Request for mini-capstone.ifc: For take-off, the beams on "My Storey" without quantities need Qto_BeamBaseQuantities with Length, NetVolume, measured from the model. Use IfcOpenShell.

First a look at what the model holds.

```python
import ifcopenshell
import ifcopenshell.util.element
import ifcopenshell.util.unit

model = ifcopenshell.open("mini-capstone.ifc")
print(model.schema)
for unit_type in ("LENGTHUNIT", "AREAUNIT", "VOLUMEUNIT"):
    print(unit_type, ifcopenshell.util.unit.calculate_unit_scale(model, unit_type))
storey = next(s for s in model.by_type("IfcBuildingStorey") if s.Name == "My Storey")
beams = [e for e in ifcopenshell.util.element.get_decomposition(storey) if e.is_a("IfcBeam")]
for e in sorted(beams, key=lambda e: e.id()):
    print(e.id(), e.is_a(), e.Name, list(ifcopenshell.util.element.get_psets(e, qtos_only=True)), sep=" | ")
```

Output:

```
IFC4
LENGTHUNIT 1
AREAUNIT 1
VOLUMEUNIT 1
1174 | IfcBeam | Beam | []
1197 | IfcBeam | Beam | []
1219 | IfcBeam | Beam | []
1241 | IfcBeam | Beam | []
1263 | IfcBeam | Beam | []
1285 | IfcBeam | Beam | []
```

```python
import ifcopenshell
import ifcopenshell.api.pset
import ifcopenshell.geom
import ifcopenshell.util.element
import ifcopenshell.util.shape
import ifcopenshell.util.unit

model = ifcopenshell.open("mini-capstone.ifc")
unit_scale = ifcopenshell.util.unit.calculate_unit_scale(model)
volume_scale = ifcopenshell.util.unit.calculate_unit_scale(model, "VOLUMEUNIT")
settings = ifcopenshell.geom.settings()

storey = next(s for s in model.by_type("IfcBuildingStorey") if s.Name == "My Storey")
beams = [e for e in ifcopenshell.util.element.get_decomposition(storey) if e.is_a("IfcBeam")]

for e in sorted(beams, key=lambda e: e.id()):
    if ifcopenshell.util.element.get_psets(e, qtos_only=True, should_inherit=False):
        continue
    # Geometry comes back in metres, in the element's own axes.
    shape = ifcopenshell.geom.create_shape(settings, e)
    values = {
        "Length": ifcopenshell.util.shape.get_max_xyz(shape.geometry) / unit_scale,
        "NetVolume": ifcopenshell.util.shape.get_volume(shape.geometry) / volume_scale,
    }
    qto = ifcopenshell.api.pset.add_qto(model, product=e, name="Qto_BeamBaseQuantities")
    ifcopenshell.api.pset.edit_qto(model, qto=qto, properties=values)
    print(e.id(), {k: round(v, 3) for k, v in values.items()})

model.write("mini-capstone-out.ifc")
```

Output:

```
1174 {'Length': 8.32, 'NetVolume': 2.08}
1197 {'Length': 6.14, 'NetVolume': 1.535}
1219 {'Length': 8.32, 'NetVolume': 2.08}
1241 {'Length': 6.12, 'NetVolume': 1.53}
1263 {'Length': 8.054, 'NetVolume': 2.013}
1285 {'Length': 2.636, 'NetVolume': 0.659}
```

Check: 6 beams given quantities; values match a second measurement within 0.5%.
